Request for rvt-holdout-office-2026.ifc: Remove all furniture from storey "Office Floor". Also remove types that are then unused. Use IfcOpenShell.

First a look at what the model holds.

```python
import ifcopenshell
import ifcopenshell.util.element

model = ifcopenshell.open("rvt-holdout-office-2026.ifc")
print(model.schema)
storey = next(s for s in model.by_type("IfcBuildingStorey") if s.Name == "Office Floor")
furniture = [e for e in ifcopenshell.util.element.get_decomposition(storey) if e.is_a("IfcFurnishingElement")]
seen = {}
for e in furniture:
    element_type = ifcopenshell.util.element.get_type(e)
    name = element_type.Name if element_type not in (None, e) else None
    seen[name] = seen.get(name, 0) + 1
for name, count in sorted(seen.items(), key=str):
    print(count, "x", name)
```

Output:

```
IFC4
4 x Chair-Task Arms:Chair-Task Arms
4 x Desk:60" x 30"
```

```python
import ifcopenshell
import ifcopenshell.api.root
import ifcopenshell.util.element

model = ifcopenshell.open("rvt-holdout-office-2026.ifc")

storey = next(s for s in model.by_type("IfcBuildingStorey") if s.Name == "Office Floor")
furniture = [e for e in ifcopenshell.util.element.get_decomposition(storey) if e.is_a("IfcFurnishingElement")]
types = {ifcopenshell.util.element.get_type(e) for e in furniture} - {None, *furniture}

for e in furniture:
    ifcopenshell.api.root.remove_product(model, product=e)
print(len(furniture), "removed")

unused = [t for t in types if not ifcopenshell.util.element.get_types(t)]
for t in unused:
    ifcopenshell.api.root.remove_product(model, product=t)
print(len(unused), "unused types removed")

model.write("rvt-holdout-office-2026_updated.ifc")
```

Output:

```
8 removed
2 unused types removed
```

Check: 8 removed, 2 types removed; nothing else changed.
